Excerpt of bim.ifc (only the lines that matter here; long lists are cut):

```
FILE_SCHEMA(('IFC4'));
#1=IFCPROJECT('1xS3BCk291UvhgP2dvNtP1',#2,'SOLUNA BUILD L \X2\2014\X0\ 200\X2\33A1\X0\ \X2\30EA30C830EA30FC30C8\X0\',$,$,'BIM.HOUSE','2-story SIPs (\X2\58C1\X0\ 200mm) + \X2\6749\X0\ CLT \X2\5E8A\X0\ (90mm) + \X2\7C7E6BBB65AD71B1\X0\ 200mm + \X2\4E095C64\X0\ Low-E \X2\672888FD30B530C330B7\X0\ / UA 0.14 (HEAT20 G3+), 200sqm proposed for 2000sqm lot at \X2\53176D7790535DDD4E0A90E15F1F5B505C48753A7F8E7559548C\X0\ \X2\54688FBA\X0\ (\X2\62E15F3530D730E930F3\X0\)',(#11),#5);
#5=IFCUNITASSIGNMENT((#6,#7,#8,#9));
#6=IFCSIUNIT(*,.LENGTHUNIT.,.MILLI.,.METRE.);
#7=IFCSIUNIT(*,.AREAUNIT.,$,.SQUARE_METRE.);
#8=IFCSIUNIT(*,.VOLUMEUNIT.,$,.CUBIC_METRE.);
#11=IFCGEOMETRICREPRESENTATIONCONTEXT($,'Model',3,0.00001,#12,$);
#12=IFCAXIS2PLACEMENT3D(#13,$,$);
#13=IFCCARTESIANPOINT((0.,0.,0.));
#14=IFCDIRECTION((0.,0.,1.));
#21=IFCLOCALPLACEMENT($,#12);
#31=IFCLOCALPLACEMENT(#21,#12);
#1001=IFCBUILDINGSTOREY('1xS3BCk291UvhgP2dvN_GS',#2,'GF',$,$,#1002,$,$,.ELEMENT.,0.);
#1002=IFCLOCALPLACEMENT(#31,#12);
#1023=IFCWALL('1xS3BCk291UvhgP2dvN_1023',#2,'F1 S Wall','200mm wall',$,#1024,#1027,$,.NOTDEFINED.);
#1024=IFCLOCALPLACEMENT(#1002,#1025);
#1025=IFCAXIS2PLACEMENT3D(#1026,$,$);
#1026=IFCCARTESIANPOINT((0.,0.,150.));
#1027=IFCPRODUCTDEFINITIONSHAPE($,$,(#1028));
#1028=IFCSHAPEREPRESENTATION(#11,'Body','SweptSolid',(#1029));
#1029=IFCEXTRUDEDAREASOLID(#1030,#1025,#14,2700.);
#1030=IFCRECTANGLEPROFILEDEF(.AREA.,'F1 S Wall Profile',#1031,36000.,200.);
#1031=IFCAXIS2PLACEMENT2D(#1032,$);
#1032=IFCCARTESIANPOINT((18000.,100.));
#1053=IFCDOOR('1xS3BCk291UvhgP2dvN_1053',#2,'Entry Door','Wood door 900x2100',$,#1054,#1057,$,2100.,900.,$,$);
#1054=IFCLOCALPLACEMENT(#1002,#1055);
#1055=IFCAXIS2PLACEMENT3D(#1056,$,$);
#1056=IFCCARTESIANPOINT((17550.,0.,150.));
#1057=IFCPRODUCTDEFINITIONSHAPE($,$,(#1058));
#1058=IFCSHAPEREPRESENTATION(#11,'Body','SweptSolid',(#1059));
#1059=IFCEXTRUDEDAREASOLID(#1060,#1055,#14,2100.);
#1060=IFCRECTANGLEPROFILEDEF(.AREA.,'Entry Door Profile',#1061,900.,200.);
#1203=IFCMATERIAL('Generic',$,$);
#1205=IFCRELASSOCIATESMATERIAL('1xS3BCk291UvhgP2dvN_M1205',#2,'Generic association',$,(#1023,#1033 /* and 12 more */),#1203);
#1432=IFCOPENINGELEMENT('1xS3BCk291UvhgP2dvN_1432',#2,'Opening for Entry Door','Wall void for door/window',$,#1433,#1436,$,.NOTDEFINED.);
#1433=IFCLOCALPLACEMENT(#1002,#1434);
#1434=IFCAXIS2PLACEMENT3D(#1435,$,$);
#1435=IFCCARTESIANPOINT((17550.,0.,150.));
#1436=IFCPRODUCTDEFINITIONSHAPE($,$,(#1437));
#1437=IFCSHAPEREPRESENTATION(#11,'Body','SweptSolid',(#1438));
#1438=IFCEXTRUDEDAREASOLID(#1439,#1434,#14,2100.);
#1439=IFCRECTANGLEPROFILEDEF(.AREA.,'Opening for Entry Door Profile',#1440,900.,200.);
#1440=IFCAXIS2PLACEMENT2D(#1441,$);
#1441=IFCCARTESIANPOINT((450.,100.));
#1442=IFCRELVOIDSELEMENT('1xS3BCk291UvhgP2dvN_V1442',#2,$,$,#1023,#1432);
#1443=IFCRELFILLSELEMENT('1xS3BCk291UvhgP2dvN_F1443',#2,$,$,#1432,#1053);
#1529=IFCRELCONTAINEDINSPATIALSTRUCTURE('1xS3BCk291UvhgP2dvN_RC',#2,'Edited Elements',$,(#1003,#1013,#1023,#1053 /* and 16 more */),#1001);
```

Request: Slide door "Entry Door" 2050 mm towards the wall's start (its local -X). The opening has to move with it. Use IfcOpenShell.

```python
import ifcopenshell
import ifcopenshell.api.geometry
import ifcopenshell.util.placement
import ifcopenshell.util.unit

model = ifcopenshell.open("bim.ifc")
unit_scale = ifcopenshell.util.unit.calculate_unit_scale(model)

door = model.by_guid("1xS3BCk291UvhgP2dvN_1053")
opening = door.FillsVoids[0].RelatingOpeningElement
wall = opening.VoidsElements[0].RelatingBuildingElement

wall_matrix = ifcopenshell.util.placement.get_local_placement(wall.ObjectPlacement)
shift = wall_matrix[:3, 0] * -2.05 / unit_scale
before = ifcopenshell.util.placement.get_local_placement(door.ObjectPlacement)[:3, 3].copy()

# The door is not placed relative to its opening, so move both.
for product in (opening, door):
    matrix = ifcopenshell.util.placement.get_local_placement(product.ObjectPlacement)
    matrix[:3, 3] += shift
    ifcopenshell.api.geometry.edit_object_placement(model, product=product, matrix=matrix, is_si=False)

after = ifcopenshell.util.placement.get_local_placement(door.ObjectPlacement)[:3, 3]
print("door moved by", (after - before).round(3) + 0.0)

model.write("bim_updated.ifc")
```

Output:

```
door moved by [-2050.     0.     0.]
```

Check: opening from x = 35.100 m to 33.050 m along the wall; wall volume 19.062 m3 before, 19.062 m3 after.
